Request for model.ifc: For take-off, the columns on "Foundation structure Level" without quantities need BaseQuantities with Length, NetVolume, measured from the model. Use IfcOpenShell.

First a look at what the model holds.

```python
import ifcopenshell
import ifcopenshell.util.element
import ifcopenshell.util.unit

model = ifcopenshell.open("model.ifc")
print(model.schema)
for unit_type in ("LENGTHUNIT", "AREAUNIT", "VOLUMEUNIT"):
    print(unit_type, ifcopenshell.util.unit.calculate_unit_scale(model, unit_type))
storey = next(s for s in model.by_type("IfcBuildingStorey") if s.Name == "Foundation structure Level")
columns = [e for e in ifcopenshell.util.element.get_decomposition(storey) if e.is_a("IfcColumn")]
for e in sorted(columns, key=lambda e: e.id()):
    print(e.id(), e.is_a(), e.Name, list(ifcopenshell.util.element.get_psets(e, qtos_only=True)), sep=" | ")
```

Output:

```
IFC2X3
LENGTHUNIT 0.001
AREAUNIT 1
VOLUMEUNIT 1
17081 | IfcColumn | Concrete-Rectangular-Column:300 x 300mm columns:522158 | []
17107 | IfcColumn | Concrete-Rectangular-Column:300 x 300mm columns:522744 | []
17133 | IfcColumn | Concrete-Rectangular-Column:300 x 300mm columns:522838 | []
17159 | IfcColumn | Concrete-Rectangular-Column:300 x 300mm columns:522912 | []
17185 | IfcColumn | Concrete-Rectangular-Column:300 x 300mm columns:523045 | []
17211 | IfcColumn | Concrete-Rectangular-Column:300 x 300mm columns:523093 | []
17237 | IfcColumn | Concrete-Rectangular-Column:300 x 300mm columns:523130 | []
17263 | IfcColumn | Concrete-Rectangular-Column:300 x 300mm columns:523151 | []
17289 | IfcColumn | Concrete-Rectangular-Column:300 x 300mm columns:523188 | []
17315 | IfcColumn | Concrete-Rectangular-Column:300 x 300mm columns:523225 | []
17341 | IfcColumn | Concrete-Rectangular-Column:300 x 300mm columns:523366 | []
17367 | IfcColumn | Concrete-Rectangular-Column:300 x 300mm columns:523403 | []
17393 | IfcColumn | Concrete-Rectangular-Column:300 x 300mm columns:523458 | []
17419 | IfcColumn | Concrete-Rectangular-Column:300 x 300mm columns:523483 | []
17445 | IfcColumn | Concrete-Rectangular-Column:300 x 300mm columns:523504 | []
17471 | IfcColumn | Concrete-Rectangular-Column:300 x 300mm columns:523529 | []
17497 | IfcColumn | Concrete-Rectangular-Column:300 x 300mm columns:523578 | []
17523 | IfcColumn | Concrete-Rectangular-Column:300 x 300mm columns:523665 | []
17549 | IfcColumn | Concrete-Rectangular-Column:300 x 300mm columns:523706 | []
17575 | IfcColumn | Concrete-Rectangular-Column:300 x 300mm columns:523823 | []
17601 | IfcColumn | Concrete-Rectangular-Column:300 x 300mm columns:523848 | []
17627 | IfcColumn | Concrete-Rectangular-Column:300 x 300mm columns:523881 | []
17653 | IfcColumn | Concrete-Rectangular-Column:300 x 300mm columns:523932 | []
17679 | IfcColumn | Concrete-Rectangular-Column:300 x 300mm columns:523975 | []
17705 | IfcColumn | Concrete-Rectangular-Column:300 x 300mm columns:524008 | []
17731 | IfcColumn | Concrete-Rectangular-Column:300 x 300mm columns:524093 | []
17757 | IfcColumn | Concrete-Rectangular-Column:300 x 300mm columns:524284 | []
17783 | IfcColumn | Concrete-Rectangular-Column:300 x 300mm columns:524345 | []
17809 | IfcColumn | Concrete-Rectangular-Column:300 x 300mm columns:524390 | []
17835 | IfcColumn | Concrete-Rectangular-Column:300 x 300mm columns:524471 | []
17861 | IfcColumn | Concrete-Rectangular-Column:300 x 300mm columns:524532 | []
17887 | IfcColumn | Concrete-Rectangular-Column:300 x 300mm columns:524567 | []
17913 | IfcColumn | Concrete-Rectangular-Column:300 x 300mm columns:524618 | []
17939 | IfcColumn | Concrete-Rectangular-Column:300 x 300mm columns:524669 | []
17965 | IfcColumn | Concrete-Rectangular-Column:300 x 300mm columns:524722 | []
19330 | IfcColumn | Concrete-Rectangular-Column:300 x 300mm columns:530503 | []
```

```python
import ifcopenshell
import ifcopenshell.api.pset
import ifcopenshell.geom
import ifcopenshell.util.element
import ifcopenshell.util.shape
import ifcopenshell.util.unit

model = ifcopenshell.open("model.ifc")
unit_scale = ifcopenshell.util.unit.calculate_unit_scale(model)
volume_scale = ifcopenshell.util.unit.calculate_unit_scale(model, "VOLUMEUNIT")
settings = ifcopenshell.geom.settings()

storey = next(s for s in model.by_type("IfcBuildingStorey") if s.Name == "Foundation structure Level")
columns = [e for e in ifcopenshell.util.element.get_decomposition(storey) if e.is_a("IfcColumn")]

for e in sorted(columns, key=lambda e: e.id()):
    if ifcopenshell.util.element.get_psets(e, qtos_only=True, should_inherit=False):
        continue
    # Geometry comes back in metres, in the element's own axes.
    shape = ifcopenshell.geom.create_shape(settings, e)
    values = {
        "Length": ifcopenshell.util.shape.get_z(shape.geometry) / unit_scale,
        "NetVolume": ifcopenshell.util.shape.get_volume(shape.geometry) / volume_scale,
    }
    qto = ifcopenshell.api.pset.add_qto(model, product=e, name="BaseQuantities")
    ifcopenshell.api.pset.edit_qto(model, qto=qto, properties=values)
    print(e.id(), {k: round(v, 3) for k, v in values.items()})

model.write("model_edited.ifc")
```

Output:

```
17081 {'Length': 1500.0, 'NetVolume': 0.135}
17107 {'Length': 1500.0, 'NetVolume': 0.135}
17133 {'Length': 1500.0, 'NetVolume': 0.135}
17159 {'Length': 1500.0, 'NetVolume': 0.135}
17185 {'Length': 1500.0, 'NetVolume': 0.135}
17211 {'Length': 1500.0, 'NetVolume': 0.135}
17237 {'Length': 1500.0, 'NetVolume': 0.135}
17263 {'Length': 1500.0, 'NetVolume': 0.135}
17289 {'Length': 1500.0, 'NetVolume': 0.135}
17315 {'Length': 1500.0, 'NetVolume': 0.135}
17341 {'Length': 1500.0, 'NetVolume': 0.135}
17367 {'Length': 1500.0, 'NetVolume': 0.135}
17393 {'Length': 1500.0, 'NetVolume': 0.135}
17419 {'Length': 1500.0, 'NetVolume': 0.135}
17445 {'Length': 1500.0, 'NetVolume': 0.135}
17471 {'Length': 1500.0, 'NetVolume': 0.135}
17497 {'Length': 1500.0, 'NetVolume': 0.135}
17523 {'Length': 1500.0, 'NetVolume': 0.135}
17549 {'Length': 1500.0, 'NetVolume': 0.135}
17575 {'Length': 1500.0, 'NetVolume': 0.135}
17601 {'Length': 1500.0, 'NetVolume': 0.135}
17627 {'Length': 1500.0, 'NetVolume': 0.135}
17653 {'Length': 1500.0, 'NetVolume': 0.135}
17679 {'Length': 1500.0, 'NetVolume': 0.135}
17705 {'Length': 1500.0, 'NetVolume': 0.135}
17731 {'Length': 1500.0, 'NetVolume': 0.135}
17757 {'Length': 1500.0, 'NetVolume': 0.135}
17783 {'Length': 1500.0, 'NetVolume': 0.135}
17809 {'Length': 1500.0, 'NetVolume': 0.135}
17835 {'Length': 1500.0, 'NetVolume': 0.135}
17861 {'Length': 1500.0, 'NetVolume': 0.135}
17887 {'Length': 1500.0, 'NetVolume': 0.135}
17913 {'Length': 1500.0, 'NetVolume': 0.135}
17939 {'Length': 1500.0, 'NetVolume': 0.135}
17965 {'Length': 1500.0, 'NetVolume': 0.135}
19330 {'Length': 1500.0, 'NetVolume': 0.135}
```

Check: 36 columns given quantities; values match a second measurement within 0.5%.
